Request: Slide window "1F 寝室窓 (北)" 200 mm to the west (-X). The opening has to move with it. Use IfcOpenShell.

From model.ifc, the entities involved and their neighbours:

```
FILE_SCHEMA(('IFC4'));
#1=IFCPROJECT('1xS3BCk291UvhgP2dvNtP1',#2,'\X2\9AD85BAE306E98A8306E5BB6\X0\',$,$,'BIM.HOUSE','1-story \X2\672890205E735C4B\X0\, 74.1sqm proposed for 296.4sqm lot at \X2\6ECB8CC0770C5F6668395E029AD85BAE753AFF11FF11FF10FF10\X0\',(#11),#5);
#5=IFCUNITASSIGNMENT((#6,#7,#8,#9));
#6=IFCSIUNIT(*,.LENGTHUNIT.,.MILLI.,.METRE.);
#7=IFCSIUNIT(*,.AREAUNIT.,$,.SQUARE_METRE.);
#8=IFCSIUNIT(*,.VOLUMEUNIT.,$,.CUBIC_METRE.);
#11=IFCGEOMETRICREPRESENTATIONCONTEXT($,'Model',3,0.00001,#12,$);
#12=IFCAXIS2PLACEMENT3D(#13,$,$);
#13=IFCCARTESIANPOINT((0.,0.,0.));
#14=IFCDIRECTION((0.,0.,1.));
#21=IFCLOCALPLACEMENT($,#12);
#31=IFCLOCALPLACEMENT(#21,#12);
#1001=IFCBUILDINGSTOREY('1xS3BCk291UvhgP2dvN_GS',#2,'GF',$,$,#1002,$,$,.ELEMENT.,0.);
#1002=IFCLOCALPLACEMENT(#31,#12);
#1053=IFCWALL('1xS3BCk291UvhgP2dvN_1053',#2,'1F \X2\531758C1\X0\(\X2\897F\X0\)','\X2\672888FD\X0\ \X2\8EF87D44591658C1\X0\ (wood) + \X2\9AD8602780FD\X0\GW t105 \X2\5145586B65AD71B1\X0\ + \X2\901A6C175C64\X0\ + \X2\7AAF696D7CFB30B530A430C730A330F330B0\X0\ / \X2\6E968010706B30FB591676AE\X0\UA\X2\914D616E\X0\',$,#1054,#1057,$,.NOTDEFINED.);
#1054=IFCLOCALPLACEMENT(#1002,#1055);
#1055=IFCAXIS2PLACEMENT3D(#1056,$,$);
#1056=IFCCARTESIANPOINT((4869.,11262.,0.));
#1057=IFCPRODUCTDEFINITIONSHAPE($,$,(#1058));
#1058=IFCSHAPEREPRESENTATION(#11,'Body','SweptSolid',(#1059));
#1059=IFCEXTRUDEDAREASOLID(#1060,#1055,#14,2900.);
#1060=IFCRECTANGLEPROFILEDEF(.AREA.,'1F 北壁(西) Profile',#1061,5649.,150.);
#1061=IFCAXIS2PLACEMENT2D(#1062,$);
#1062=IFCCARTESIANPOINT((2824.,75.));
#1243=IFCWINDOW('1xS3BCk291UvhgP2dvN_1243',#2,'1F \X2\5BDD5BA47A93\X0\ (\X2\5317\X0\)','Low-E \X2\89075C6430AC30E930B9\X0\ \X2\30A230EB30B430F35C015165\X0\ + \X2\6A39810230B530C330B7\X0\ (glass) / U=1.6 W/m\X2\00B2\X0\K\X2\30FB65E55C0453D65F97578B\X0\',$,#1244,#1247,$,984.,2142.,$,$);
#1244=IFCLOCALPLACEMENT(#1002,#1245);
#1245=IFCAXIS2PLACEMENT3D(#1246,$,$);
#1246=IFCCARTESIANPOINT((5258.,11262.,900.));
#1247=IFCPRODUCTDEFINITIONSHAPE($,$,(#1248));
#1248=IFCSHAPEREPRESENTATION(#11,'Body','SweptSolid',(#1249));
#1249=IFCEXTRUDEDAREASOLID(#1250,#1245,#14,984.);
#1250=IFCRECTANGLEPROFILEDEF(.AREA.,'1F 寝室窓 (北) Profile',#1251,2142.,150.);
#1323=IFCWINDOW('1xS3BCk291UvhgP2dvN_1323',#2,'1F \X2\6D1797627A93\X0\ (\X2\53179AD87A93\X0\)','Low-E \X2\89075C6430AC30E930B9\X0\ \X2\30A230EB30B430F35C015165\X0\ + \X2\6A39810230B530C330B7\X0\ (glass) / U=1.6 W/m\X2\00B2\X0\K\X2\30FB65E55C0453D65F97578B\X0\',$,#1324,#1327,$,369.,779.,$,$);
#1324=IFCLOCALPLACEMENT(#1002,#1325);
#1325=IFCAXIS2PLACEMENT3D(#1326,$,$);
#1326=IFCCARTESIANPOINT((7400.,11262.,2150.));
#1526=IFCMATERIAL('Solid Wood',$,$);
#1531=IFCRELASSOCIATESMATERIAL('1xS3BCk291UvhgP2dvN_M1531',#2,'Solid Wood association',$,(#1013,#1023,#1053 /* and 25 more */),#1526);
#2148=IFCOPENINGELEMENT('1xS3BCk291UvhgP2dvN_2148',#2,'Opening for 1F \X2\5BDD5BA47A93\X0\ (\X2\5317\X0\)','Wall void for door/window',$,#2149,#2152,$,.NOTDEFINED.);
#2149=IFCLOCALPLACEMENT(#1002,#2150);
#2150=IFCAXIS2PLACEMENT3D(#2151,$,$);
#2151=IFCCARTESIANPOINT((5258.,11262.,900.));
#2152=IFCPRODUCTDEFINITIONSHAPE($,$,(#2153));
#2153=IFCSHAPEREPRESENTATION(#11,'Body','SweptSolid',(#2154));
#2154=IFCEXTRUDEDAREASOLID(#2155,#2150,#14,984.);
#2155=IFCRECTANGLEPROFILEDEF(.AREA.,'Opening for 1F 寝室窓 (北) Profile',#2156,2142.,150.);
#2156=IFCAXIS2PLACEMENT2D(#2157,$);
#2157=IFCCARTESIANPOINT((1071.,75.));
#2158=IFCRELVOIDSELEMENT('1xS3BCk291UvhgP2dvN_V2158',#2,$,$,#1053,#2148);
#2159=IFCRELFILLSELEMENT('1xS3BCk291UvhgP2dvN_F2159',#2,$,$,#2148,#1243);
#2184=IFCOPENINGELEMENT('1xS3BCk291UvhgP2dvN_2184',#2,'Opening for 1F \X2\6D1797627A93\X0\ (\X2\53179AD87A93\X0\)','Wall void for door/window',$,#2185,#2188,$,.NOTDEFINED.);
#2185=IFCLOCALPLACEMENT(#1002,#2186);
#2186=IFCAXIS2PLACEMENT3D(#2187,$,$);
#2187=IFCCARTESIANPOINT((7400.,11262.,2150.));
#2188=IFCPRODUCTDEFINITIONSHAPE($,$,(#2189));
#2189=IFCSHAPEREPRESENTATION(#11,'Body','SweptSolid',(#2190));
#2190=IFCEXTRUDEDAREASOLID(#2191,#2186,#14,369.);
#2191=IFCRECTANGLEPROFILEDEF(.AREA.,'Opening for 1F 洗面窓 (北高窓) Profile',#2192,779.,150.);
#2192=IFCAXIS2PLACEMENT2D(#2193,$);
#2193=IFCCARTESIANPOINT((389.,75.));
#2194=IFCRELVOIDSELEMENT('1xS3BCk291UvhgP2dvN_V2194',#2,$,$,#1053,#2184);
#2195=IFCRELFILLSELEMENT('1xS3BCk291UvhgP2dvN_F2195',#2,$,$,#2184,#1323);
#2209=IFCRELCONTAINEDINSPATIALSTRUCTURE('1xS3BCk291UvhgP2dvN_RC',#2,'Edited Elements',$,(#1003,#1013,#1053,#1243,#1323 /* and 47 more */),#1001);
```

```python
import ifcopenshell
import ifcopenshell.api.geometry
import ifcopenshell.util.placement

model = ifcopenshell.open("model.ifc")

window = model.by_guid("1xS3BCk291UvhgP2dvN_1243")
opening = window.FillsVoids[0].RelatingOpeningElement
wall = opening.VoidsElements[0].RelatingBuildingElement

wall_matrix = ifcopenshell.util.placement.get_local_placement(wall.ObjectPlacement)
shift = wall_matrix[:3, 0] * -200.0
before = ifcopenshell.util.placement.get_local_placement(window.ObjectPlacement)[:3, 3].copy()

# The window is not placed relative to its opening, so move both.
for product in (opening, window):
    matrix = ifcopenshell.util.placement.get_local_placement(product.ObjectPlacement)
    matrix[:3, 3] += shift
    ifcopenshell.api.geometry.edit_object_placement(model, product=product, matrix=matrix, is_si=False)

after = ifcopenshell.util.placement.get_local_placement(window.ObjectPlacement)[:3, 3]
print("window moved by", (after - before).round(3) + 0.0)

model.write("model_rev.ifc")
```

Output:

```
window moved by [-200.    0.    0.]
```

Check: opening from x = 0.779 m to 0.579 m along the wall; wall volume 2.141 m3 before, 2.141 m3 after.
